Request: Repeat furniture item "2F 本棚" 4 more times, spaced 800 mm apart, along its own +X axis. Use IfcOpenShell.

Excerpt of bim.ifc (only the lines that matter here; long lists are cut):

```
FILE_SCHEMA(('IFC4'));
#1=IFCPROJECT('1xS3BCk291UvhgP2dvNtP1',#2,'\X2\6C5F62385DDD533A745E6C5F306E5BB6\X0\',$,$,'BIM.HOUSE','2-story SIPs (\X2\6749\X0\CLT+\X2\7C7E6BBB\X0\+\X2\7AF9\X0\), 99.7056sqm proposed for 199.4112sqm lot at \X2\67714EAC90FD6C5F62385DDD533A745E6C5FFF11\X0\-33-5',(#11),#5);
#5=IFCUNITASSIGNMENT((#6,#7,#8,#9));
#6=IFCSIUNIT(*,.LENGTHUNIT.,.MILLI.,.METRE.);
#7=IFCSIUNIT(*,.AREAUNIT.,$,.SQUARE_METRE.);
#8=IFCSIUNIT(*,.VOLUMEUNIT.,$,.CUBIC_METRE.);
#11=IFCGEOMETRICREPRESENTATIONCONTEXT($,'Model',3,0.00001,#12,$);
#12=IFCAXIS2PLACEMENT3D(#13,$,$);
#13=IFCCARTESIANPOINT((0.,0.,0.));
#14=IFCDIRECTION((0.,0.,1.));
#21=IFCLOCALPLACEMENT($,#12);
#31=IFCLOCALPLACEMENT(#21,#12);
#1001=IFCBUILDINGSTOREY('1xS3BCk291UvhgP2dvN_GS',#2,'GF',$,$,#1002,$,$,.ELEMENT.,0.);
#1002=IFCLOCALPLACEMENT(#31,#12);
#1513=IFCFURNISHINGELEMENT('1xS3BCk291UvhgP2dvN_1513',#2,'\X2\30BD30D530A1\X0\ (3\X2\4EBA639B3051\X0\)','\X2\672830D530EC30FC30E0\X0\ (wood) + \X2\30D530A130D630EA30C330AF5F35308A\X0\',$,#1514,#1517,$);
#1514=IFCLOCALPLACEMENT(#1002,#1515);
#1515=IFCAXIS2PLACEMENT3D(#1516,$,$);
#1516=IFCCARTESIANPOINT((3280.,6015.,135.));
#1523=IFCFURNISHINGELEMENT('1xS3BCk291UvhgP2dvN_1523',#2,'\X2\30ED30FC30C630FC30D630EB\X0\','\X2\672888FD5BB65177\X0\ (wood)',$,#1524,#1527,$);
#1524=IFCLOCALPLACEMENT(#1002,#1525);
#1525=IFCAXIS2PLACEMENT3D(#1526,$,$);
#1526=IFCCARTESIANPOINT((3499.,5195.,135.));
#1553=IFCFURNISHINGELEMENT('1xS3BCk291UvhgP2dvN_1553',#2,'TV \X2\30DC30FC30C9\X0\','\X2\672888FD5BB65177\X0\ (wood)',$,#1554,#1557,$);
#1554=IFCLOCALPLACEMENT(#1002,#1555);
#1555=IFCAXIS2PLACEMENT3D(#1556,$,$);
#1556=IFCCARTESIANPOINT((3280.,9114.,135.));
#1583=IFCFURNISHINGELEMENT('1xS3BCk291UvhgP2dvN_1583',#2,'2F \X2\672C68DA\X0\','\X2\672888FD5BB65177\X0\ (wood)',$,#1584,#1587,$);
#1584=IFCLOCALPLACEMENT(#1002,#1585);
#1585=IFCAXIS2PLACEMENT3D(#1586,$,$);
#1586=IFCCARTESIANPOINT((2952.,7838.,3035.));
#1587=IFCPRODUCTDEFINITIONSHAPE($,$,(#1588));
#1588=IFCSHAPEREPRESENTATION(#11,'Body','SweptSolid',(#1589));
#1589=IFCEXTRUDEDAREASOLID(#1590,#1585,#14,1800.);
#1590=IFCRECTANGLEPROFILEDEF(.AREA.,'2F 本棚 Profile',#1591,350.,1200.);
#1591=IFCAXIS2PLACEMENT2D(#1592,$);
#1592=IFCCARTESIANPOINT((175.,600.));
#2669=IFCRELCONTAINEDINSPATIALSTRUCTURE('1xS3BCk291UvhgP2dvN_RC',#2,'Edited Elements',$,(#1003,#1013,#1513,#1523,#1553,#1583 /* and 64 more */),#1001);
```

```python
import ifcopenshell
import ifcopenshell.api.geometry
import ifcopenshell.api.root
import ifcopenshell.util.element
import ifcopenshell.util.placement
import ifcopenshell.util.unit

model = ifcopenshell.open("bim.ifc")
unit_scale = ifcopenshell.util.unit.calculate_unit_scale(model)


def reuse_history(source, copy):
    """copy_class also copies each property set's owner history, people and application; keep the originals."""
    for rel in copy.IsDefinedBy:
        if rel.is_a("IfcRelDefinesByProperties") and (history := rel.RelatingPropertyDefinition.OwnerHistory):
            rel.RelatingPropertyDefinition.OwnerHistory = source.OwnerHistory
            ifcopenshell.util.element.remove_deep2(model, history)


source = model.by_guid("1xS3BCk291UvhgP2dvN_1583")
base = ifcopenshell.util.placement.get_local_placement(source.ObjectPlacement)
step = base[:3, 0] * 0.8 / unit_scale

for i in range(1, 5):
    copy = ifcopenshell.api.root.copy_class(model, product=source)
    copy.Representation = ifcopenshell.util.element.copy_deep(
        model, source.Representation, exclude=["IfcGeometricRepresentationContext", "IfcRepresentationMap"]
    )
    reuse_history(source, copy)
    matrix = base.copy()
    matrix[:3, 3] += i * step
    print("added at", matrix[:3, 3].round(3) + 0.0)
    ifcopenshell.api.geometry.edit_object_placement(model, product=copy, matrix=matrix, is_si=False)

model.write("bim_v2.ifc")
```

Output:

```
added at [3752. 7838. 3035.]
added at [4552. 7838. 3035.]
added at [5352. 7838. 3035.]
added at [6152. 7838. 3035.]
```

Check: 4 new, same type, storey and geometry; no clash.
